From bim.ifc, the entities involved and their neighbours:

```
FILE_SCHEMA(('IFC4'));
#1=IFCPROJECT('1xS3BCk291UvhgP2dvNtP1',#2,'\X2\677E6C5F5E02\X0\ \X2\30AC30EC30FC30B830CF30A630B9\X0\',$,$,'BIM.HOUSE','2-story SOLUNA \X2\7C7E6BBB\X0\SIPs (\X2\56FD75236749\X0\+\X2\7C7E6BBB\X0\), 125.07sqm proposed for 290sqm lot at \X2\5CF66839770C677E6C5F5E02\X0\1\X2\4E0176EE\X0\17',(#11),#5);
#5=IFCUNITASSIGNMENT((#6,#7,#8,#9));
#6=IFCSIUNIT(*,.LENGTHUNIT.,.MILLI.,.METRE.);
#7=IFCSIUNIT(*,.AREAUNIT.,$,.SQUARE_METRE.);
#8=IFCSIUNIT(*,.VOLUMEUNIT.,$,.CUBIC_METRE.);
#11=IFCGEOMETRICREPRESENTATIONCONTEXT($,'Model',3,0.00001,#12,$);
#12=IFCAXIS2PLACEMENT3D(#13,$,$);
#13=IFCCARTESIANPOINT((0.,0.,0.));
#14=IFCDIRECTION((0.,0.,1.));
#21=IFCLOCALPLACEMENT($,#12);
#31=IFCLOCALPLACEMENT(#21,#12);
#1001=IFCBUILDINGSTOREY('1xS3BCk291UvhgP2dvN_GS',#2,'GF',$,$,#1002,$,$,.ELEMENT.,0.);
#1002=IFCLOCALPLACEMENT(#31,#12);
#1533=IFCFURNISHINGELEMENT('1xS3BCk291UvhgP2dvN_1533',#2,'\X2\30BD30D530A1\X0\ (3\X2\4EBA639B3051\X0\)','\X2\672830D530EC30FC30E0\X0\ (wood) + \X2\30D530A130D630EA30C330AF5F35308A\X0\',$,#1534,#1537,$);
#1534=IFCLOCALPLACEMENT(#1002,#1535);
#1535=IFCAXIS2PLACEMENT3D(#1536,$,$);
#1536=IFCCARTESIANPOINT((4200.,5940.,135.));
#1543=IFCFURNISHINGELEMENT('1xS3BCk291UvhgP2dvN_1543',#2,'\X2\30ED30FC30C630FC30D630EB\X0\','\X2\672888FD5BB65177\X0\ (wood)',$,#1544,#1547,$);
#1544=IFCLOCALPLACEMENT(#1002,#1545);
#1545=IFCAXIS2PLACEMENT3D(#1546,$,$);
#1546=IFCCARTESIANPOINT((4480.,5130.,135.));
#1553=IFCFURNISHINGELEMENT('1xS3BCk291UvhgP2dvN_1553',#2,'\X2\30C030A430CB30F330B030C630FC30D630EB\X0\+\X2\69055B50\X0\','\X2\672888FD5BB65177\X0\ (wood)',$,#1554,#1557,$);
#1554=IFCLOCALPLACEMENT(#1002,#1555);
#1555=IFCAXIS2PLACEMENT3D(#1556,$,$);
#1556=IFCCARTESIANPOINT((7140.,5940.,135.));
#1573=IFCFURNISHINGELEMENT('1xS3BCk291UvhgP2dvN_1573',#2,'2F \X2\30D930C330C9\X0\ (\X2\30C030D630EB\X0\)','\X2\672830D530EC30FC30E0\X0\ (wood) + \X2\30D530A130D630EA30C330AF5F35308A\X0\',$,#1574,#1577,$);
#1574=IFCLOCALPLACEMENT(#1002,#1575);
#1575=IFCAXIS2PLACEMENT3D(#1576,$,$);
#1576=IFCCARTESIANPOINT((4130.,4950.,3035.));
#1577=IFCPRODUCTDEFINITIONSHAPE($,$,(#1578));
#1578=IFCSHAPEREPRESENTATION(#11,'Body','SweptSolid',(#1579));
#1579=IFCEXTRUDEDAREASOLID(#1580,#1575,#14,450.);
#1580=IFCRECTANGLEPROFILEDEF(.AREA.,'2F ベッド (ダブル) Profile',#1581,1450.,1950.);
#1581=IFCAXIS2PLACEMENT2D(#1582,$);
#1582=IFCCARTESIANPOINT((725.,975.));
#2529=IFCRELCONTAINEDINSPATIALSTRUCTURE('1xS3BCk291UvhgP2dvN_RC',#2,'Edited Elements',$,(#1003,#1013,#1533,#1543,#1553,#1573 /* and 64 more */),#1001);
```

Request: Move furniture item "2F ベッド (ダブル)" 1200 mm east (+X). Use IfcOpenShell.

```python
import ifcopenshell
import ifcopenshell.api.geometry
import ifcopenshell.util.placement
import ifcopenshell.util.unit

model = ifcopenshell.open("bim.ifc")
unit_scale = ifcopenshell.util.unit.calculate_unit_scale(model)

item = model.by_id(1573)
matrix = ifcopenshell.util.placement.get_local_placement(item.ObjectPlacement)
matrix[0, 3] += 1.2 / unit_scale
ifcopenshell.api.geometry.edit_object_placement(model, product=item, matrix=matrix, is_si=False)

print(ifcopenshell.util.placement.get_local_placement(item.ObjectPlacement).round(3) + 0.0)

model.write("bim_v2.ifc")
```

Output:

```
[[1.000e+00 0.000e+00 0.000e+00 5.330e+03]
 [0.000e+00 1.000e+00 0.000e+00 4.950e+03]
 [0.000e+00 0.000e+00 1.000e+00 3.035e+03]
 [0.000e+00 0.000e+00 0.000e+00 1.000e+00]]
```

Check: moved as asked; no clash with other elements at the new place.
